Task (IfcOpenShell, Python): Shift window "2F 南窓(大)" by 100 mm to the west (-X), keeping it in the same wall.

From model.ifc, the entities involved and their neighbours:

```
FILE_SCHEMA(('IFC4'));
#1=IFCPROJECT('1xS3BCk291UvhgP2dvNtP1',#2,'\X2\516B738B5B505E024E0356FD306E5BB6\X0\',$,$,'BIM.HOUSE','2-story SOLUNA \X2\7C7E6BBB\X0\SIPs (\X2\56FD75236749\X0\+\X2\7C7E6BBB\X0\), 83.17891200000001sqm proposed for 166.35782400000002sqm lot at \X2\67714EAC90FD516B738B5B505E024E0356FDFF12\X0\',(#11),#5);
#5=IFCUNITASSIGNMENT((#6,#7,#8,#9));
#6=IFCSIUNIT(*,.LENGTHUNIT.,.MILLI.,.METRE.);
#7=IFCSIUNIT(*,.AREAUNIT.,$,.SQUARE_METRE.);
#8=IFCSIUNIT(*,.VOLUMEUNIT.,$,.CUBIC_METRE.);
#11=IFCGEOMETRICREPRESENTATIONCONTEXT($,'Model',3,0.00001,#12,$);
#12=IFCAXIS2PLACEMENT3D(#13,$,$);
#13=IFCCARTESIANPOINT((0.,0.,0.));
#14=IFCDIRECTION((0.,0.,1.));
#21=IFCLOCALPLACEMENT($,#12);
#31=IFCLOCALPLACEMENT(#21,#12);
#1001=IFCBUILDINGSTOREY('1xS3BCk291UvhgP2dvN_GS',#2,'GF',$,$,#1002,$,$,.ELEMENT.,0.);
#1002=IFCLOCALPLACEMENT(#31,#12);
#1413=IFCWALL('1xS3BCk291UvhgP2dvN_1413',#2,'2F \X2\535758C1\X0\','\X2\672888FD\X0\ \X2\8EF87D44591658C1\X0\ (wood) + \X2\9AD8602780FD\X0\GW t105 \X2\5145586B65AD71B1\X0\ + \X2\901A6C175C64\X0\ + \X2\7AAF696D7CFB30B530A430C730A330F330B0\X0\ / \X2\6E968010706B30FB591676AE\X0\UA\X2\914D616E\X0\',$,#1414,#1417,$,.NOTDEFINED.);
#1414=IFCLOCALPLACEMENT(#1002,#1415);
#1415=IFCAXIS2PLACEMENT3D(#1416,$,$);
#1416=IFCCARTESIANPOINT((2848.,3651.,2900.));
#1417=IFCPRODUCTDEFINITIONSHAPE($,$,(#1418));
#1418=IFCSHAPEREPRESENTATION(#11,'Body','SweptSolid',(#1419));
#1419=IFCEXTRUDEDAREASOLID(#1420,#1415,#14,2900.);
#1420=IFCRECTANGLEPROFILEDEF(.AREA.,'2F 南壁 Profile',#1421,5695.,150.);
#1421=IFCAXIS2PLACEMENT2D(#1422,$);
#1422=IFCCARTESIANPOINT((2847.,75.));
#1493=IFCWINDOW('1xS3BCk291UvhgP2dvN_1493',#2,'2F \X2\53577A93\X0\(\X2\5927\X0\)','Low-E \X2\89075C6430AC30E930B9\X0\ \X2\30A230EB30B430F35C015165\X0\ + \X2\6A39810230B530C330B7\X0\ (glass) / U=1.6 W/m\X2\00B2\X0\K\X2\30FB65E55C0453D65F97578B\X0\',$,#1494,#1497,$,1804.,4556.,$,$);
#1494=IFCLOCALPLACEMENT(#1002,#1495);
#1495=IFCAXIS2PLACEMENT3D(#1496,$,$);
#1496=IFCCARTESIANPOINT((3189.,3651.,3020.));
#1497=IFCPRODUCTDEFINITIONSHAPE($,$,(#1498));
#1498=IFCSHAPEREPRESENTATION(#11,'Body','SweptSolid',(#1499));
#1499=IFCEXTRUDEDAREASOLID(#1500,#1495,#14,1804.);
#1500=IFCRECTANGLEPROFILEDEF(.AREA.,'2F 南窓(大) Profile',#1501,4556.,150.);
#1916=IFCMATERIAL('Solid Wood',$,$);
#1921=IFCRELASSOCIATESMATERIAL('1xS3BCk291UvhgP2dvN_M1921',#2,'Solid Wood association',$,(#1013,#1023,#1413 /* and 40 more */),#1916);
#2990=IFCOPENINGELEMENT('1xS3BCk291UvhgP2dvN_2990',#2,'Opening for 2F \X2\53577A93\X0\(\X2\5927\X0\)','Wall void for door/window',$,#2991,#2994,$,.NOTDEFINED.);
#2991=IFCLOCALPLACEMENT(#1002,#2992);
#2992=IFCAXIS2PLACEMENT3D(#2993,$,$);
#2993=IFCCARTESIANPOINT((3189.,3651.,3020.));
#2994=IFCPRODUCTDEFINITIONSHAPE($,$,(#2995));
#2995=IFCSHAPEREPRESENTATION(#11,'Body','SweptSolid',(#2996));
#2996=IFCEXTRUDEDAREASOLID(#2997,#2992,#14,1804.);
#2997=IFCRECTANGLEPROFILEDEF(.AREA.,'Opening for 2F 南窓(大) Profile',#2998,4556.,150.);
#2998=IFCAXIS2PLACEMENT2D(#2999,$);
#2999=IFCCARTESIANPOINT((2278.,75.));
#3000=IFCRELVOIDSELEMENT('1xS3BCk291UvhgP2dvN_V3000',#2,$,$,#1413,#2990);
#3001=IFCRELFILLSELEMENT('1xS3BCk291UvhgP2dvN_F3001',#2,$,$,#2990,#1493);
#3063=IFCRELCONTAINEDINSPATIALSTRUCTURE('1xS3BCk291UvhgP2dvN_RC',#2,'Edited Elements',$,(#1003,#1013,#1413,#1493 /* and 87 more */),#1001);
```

```python
import ifcopenshell
import ifcopenshell.api.geometry
import ifcopenshell.util.placement

model = ifcopenshell.open("model.ifc")

window = model.by_id(1493)
opening = window.FillsVoids[0].RelatingOpeningElement
wall = opening.VoidsElements[0].RelatingBuildingElement

wall_matrix = ifcopenshell.util.placement.get_local_placement(wall.ObjectPlacement)
shift = wall_matrix[:3, 0] * -100.0
before = ifcopenshell.util.placement.get_local_placement(window.ObjectPlacement)[:3, 3].copy()

# The window is not placed relative to its opening, so move both.
for product in (opening, window):
    matrix = ifcopenshell.util.placement.get_local_placement(product.ObjectPlacement)
    matrix[:3, 3] += shift
    ifcopenshell.api.geometry.edit_object_placement(model, product=product, matrix=matrix, is_si=False)

after = ifcopenshell.util.placement.get_local_placement(window.ObjectPlacement)[:3, 3]
print("window moved by", (after - before).round(3) + 0.0)

model.write("model-out.ifc")
```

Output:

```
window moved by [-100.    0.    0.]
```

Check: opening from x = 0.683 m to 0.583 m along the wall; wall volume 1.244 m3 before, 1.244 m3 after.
